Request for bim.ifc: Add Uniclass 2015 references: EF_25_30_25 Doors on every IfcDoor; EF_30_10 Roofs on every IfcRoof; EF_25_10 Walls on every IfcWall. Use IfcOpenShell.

First a look at what the model holds.

```python
import ifcopenshell

model = ifcopenshell.open("bim.ifc")
print(model.schema)
print("classifications:", [c.Name for c in model.by_type("IfcClassification")])
for ifc_class in ("IfcDoor", "IfcRoof", "IfcStair", "IfcWall", "IfcWindow"):
    print(ifc_class, len(model.by_type(ifc_class)))
```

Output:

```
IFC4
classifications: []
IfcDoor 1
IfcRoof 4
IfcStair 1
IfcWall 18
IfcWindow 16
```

```python
import ifcopenshell
import ifcopenshell.api.classification

model = ifcopenshell.open("bim.ifc")

system = ifcopenshell.api.classification.add_classification(model, classification="Uniclass 2015")

codes = {
    "IfcDoor": ("EF_25_30_25", "Doors"),
    "IfcRoof": ("EF_30_10", "Roofs"),
    "IfcWall": ("EF_25_10", "Walls"),
}
for ifc_class, (code, name) in codes.items():
    products = model.by_type(ifc_class)
    ifcopenshell.api.classification.add_reference(
        model, products=products, classification=system, identification=code, name=name
    )
    print(code, len(products))

model.write("bim_updated.ifc")
```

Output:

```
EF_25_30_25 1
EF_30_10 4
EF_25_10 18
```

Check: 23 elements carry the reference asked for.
